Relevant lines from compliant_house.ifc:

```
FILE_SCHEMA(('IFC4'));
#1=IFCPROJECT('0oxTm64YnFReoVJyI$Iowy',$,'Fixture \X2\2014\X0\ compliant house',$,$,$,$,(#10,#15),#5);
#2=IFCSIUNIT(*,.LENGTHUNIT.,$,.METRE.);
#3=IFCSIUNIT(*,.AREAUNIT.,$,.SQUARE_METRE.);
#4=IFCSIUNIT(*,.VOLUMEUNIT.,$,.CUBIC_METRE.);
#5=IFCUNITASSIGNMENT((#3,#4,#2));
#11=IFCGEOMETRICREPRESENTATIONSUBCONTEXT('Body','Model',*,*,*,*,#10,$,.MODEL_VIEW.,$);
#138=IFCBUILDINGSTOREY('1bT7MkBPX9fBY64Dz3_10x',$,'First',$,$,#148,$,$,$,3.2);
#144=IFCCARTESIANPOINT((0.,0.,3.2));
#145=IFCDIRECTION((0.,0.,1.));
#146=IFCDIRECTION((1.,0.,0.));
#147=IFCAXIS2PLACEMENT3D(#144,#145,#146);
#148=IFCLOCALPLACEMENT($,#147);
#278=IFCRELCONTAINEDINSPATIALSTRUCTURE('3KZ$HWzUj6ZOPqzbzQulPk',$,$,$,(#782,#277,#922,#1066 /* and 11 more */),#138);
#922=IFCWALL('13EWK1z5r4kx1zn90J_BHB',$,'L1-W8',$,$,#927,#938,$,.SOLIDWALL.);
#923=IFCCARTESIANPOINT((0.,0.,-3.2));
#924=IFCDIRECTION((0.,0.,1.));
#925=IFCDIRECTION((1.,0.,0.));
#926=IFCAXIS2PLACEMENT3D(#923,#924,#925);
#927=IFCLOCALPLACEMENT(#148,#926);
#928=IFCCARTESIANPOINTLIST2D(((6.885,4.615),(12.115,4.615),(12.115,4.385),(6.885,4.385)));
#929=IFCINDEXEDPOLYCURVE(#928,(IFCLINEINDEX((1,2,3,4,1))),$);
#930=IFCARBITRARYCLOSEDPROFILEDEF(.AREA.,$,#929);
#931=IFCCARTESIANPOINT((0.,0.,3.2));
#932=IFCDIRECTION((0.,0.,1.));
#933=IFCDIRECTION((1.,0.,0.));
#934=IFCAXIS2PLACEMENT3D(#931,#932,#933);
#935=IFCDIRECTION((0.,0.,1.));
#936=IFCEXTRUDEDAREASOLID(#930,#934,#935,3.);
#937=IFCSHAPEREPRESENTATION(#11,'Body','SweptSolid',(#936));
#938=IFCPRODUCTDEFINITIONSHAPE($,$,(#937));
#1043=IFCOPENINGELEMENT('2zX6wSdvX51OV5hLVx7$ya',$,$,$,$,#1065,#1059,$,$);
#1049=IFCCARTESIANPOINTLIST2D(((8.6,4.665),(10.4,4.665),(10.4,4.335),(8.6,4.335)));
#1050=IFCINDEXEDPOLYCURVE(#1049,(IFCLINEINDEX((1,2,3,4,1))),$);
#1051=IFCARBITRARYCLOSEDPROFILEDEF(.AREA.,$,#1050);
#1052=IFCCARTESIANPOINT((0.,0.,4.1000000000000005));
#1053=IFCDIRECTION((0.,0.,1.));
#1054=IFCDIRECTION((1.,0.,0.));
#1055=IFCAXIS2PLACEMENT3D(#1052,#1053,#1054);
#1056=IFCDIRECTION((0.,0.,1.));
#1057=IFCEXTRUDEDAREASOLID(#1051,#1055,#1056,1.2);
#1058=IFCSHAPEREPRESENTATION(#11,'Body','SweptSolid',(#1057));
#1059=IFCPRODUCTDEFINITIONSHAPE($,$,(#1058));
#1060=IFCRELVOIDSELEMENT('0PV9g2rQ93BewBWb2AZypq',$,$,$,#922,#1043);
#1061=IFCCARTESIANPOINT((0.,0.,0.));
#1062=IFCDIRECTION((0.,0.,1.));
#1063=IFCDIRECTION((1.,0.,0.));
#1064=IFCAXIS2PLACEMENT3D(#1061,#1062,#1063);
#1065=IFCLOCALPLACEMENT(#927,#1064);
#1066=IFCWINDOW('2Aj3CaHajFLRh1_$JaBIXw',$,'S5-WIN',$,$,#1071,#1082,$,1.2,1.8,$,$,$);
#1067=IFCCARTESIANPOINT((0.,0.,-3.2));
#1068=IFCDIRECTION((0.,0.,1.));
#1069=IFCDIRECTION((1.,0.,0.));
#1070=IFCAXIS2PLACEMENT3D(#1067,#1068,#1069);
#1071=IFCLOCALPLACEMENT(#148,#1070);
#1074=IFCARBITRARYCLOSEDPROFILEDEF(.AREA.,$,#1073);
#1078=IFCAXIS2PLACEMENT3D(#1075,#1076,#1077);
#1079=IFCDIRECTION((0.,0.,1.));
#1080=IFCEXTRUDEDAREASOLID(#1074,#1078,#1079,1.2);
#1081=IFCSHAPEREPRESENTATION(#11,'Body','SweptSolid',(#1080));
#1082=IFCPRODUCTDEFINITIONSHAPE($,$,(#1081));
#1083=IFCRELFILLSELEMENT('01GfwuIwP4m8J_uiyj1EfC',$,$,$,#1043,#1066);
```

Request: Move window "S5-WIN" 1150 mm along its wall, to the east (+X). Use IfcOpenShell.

```python
import ifcopenshell
import ifcopenshell.api.geometry
import ifcopenshell.util.placement
import ifcopenshell.util.unit

model = ifcopenshell.open("compliant_house.ifc")
unit_scale = ifcopenshell.util.unit.calculate_unit_scale(model)

window = model.by_guid("2Aj3CaHajFLRh1_$JaBIXw")
opening = window.FillsVoids[0].RelatingOpeningElement
wall = opening.VoidsElements[0].RelatingBuildingElement

wall_matrix = ifcopenshell.util.placement.get_local_placement(wall.ObjectPlacement)
shift = wall_matrix[:3, 0] * 1.15 / unit_scale
before = ifcopenshell.util.placement.get_local_placement(window.ObjectPlacement)[:3, 3].copy()

# The window is not placed relative to its opening, so move both.
for product in (opening, window):
    matrix = ifcopenshell.util.placement.get_local_placement(product.ObjectPlacement)
    matrix[:3, 3] += shift
    ifcopenshell.api.geometry.edit_object_placement(model, product=product, matrix=matrix, is_si=False)

after = ifcopenshell.util.placement.get_local_placement(window.ObjectPlacement)[:3, 3]
print("window moved by", (after - before).round(3) + 0.0)

model.write("compliant_house-out.ifc")
```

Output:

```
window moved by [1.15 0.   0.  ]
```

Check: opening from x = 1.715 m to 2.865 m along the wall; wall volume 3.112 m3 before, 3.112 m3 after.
